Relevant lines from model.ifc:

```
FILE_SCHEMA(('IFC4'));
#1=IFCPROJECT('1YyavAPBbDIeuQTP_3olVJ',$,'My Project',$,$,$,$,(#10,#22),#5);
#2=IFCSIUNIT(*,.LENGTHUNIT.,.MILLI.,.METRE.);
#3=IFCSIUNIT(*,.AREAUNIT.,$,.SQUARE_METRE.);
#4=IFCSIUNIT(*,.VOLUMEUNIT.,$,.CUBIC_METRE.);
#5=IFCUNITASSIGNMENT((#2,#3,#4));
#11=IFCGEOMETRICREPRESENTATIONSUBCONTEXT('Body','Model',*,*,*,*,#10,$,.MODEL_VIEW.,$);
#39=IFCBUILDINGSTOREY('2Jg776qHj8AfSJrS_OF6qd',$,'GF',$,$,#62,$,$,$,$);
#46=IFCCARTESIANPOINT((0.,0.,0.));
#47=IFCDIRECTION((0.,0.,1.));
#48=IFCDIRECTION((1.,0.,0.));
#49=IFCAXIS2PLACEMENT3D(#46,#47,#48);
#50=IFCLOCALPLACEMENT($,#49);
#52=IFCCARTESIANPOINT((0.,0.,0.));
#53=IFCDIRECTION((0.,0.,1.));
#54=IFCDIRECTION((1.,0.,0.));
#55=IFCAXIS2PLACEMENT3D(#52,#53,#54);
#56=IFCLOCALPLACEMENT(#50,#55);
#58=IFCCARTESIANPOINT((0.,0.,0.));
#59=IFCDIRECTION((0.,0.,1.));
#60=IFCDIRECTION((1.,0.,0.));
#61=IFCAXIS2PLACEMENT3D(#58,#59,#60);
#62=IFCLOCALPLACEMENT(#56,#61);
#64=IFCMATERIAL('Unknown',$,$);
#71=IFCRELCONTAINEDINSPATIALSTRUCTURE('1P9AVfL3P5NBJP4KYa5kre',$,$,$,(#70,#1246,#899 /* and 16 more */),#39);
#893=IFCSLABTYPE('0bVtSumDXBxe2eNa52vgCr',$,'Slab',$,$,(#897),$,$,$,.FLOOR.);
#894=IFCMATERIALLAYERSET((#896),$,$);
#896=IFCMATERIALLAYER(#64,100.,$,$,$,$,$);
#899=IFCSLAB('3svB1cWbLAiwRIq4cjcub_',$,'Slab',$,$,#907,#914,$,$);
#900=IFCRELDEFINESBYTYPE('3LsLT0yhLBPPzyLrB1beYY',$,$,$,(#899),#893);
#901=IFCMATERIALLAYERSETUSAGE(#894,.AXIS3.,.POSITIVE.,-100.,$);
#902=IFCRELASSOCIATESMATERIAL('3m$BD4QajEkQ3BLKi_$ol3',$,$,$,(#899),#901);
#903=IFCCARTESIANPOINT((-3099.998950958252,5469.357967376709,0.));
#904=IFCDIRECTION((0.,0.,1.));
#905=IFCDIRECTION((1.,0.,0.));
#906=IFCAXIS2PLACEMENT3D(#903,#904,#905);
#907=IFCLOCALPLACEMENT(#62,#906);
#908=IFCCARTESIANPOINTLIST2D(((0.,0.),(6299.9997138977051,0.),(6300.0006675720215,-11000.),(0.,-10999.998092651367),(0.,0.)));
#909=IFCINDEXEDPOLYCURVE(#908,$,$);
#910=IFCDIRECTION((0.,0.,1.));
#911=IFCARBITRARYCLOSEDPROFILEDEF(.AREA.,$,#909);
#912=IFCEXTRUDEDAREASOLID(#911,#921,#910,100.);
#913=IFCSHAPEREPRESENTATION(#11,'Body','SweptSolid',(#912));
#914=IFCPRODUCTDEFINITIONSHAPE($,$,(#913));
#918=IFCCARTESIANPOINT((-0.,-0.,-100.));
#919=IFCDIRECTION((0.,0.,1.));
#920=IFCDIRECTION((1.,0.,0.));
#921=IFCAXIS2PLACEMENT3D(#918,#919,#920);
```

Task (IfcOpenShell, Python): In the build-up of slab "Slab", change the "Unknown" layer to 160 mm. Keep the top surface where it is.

```python
import ifcopenshell
import ifcopenshell.util.element
import ifcopenshell.util.representation
import ifcopenshell.util.unit

model = ifcopenshell.open("model.ifc")
unit_scale = ifcopenshell.util.unit.calculate_unit_scale(model)

layer_set = model.by_id(894)
layer = next(l for l in layer_set.MaterialLayers if l.Material and l.Material.Name == "Unknown")
change = 0.16 / unit_scale - layer.LayerThickness
layer.LayerThickness += change

# Geometry does not follow the layer set by itself.
slabs = [e for e in ifcopenshell.util.element.get_elements_by_material(model, layer_set) if e.is_a("IfcSlab")]
for slab in sorted(slabs, key=lambda e: e.id()):
    body = ifcopenshell.util.representation.get_representation(slab, "Model", "Body")
    solid = body.Items[0]
    old_depth = solid.Depth
    solid.Depth += change
    # Extruded upwards: lower the start of the extrusion so the top stays.
    x, y, z = solid.Position.Location.Coordinates
    solid.Position.Location = model.createIfcCartesianPoint((x, y, z - change))
    print(slab.id(), f"{old_depth:g} -> {solid.Depth:g}")

# The layers are counted up from the underside, which has moved.
for usage in {ifcopenshell.util.element.get_material(slab) for slab in slabs}:
    usage.OffsetFromReferenceLine -= change

model.write("model_rev.ifc")
```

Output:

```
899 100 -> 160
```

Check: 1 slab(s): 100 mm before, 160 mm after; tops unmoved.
